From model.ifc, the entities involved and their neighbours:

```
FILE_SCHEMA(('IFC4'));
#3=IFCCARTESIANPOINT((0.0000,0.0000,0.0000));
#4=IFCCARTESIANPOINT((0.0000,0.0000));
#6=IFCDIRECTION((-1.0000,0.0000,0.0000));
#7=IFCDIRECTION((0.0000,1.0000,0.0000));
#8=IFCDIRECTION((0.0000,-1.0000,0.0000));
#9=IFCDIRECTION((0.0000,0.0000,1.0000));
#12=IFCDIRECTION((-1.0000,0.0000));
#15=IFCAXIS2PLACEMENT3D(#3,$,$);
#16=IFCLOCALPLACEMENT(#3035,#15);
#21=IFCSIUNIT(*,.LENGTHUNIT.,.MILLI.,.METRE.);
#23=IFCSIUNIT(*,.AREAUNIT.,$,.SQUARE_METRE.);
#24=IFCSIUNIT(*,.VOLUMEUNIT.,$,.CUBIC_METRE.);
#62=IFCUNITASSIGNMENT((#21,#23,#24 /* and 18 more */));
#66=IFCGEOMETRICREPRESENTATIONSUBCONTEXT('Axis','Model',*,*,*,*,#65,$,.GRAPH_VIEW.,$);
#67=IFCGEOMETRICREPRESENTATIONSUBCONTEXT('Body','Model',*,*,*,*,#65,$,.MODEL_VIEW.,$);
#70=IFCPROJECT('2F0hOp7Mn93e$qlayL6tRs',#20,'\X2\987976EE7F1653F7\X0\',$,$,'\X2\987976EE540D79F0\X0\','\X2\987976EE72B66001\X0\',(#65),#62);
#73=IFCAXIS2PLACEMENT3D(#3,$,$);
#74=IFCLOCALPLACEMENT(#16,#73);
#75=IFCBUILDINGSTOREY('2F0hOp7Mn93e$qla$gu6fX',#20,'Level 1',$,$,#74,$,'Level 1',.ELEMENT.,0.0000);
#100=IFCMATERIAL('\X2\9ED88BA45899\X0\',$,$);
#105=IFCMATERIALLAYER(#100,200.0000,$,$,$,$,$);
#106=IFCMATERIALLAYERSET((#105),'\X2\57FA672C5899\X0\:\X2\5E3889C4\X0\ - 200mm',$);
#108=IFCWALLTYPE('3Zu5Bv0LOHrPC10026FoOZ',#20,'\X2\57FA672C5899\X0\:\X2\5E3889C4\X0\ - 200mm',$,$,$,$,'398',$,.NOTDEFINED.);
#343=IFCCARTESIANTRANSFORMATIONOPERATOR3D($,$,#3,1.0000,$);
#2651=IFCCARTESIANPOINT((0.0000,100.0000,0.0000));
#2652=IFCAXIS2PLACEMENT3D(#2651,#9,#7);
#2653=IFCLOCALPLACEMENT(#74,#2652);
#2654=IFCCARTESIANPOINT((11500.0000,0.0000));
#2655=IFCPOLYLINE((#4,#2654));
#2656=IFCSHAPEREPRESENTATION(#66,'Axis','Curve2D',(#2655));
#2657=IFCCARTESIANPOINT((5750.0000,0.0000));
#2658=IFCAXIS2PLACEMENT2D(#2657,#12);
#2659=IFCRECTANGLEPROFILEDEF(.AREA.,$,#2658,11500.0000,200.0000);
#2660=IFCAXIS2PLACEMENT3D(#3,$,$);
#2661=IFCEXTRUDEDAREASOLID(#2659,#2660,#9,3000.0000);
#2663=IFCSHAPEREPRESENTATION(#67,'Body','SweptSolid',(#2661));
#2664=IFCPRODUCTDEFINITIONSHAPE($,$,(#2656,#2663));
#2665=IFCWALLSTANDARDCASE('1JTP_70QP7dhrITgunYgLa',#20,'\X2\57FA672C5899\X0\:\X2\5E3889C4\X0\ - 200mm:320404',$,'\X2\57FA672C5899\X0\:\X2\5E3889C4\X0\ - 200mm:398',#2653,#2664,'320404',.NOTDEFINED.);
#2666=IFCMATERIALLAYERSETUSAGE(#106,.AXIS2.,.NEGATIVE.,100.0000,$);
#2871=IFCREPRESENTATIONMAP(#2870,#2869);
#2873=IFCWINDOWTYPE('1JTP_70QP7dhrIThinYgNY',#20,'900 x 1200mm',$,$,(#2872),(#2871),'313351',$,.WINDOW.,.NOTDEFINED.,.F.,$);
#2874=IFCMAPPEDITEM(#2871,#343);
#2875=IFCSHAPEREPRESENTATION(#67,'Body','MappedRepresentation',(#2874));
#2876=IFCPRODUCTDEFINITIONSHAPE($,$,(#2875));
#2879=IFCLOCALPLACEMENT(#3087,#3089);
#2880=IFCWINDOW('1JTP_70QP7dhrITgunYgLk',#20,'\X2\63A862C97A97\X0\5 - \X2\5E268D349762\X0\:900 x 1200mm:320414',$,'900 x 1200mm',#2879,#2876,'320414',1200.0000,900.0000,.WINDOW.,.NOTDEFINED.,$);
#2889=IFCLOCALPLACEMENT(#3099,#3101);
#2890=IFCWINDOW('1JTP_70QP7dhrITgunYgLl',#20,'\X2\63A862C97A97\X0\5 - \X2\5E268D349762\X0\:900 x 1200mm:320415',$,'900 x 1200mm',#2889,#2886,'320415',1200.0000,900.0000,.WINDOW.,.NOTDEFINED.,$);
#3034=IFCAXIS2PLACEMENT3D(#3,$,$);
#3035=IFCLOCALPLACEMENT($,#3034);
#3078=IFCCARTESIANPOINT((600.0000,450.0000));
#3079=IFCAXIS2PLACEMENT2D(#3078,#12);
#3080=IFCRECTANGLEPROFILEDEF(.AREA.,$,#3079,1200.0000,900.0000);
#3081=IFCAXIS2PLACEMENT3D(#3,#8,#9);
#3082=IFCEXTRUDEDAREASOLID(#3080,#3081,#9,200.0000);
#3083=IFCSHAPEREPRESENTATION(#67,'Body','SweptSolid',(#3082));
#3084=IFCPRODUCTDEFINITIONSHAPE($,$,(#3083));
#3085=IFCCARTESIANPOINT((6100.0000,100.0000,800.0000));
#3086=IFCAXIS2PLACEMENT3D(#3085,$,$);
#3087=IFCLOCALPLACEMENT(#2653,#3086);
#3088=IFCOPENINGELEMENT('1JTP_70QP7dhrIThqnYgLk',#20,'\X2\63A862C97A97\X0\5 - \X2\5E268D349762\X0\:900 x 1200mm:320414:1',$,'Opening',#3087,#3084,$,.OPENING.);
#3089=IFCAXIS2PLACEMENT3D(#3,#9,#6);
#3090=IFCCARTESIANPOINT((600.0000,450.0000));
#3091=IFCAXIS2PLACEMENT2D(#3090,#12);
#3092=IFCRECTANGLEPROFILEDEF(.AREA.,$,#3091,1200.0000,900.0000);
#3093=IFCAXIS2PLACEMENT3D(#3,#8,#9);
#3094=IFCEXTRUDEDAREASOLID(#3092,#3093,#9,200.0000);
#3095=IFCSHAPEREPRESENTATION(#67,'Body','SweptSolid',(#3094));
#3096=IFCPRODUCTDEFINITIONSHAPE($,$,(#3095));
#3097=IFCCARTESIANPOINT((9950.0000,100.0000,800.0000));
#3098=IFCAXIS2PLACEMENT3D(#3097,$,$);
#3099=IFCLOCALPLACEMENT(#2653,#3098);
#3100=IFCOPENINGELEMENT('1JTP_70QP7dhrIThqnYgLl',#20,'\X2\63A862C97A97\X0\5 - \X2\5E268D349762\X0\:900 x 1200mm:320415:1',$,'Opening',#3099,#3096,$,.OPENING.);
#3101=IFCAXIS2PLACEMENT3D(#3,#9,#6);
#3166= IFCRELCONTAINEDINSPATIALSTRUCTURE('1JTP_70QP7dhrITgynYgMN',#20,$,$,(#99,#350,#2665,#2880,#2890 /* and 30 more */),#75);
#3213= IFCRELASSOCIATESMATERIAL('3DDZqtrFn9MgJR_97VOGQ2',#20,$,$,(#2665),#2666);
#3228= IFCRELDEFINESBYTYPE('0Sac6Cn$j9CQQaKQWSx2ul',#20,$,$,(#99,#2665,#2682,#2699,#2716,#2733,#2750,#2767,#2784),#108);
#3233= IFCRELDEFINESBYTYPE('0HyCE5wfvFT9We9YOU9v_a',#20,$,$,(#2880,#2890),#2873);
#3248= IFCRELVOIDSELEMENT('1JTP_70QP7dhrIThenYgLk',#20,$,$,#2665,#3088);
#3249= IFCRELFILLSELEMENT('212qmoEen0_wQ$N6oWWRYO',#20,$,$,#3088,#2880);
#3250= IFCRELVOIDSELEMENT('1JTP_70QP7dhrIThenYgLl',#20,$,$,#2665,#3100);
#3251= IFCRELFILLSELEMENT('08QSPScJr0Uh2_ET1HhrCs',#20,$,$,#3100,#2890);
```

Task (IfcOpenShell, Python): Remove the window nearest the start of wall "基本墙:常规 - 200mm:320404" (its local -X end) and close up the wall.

```python
import ifcopenshell
import ifcopenshell.api.feature
import ifcopenshell.api.root
import ifcopenshell.geom
import ifcopenshell.util.shape

model = ifcopenshell.open("model.ifc")
settings = ifcopenshell.geom.settings()


def volume(element):
    """Net volume in cubic metres, openings subtracted."""
    shape = ifcopenshell.geom.create_shape(settings, element)
    return ifcopenshell.util.shape.get_volume(shape.geometry)


window = model.by_guid("1JTP_70QP7dhrITgunYgLk")
opening = window.FillsVoids[0].RelatingOpeningElement
wall = opening.VoidsElements[0].RelatingBuildingElement
before = volume(wall)

ifcopenshell.api.root.remove_product(model, product=window)
ifcopenshell.api.feature.remove_feature(model, feature=opening)

after = volume(wall)

print(f"wall volume {before:.3f} -> {after:.3f} m3")

model.write("model_v2.ifc")
```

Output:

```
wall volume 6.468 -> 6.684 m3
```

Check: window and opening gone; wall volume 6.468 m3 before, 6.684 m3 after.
